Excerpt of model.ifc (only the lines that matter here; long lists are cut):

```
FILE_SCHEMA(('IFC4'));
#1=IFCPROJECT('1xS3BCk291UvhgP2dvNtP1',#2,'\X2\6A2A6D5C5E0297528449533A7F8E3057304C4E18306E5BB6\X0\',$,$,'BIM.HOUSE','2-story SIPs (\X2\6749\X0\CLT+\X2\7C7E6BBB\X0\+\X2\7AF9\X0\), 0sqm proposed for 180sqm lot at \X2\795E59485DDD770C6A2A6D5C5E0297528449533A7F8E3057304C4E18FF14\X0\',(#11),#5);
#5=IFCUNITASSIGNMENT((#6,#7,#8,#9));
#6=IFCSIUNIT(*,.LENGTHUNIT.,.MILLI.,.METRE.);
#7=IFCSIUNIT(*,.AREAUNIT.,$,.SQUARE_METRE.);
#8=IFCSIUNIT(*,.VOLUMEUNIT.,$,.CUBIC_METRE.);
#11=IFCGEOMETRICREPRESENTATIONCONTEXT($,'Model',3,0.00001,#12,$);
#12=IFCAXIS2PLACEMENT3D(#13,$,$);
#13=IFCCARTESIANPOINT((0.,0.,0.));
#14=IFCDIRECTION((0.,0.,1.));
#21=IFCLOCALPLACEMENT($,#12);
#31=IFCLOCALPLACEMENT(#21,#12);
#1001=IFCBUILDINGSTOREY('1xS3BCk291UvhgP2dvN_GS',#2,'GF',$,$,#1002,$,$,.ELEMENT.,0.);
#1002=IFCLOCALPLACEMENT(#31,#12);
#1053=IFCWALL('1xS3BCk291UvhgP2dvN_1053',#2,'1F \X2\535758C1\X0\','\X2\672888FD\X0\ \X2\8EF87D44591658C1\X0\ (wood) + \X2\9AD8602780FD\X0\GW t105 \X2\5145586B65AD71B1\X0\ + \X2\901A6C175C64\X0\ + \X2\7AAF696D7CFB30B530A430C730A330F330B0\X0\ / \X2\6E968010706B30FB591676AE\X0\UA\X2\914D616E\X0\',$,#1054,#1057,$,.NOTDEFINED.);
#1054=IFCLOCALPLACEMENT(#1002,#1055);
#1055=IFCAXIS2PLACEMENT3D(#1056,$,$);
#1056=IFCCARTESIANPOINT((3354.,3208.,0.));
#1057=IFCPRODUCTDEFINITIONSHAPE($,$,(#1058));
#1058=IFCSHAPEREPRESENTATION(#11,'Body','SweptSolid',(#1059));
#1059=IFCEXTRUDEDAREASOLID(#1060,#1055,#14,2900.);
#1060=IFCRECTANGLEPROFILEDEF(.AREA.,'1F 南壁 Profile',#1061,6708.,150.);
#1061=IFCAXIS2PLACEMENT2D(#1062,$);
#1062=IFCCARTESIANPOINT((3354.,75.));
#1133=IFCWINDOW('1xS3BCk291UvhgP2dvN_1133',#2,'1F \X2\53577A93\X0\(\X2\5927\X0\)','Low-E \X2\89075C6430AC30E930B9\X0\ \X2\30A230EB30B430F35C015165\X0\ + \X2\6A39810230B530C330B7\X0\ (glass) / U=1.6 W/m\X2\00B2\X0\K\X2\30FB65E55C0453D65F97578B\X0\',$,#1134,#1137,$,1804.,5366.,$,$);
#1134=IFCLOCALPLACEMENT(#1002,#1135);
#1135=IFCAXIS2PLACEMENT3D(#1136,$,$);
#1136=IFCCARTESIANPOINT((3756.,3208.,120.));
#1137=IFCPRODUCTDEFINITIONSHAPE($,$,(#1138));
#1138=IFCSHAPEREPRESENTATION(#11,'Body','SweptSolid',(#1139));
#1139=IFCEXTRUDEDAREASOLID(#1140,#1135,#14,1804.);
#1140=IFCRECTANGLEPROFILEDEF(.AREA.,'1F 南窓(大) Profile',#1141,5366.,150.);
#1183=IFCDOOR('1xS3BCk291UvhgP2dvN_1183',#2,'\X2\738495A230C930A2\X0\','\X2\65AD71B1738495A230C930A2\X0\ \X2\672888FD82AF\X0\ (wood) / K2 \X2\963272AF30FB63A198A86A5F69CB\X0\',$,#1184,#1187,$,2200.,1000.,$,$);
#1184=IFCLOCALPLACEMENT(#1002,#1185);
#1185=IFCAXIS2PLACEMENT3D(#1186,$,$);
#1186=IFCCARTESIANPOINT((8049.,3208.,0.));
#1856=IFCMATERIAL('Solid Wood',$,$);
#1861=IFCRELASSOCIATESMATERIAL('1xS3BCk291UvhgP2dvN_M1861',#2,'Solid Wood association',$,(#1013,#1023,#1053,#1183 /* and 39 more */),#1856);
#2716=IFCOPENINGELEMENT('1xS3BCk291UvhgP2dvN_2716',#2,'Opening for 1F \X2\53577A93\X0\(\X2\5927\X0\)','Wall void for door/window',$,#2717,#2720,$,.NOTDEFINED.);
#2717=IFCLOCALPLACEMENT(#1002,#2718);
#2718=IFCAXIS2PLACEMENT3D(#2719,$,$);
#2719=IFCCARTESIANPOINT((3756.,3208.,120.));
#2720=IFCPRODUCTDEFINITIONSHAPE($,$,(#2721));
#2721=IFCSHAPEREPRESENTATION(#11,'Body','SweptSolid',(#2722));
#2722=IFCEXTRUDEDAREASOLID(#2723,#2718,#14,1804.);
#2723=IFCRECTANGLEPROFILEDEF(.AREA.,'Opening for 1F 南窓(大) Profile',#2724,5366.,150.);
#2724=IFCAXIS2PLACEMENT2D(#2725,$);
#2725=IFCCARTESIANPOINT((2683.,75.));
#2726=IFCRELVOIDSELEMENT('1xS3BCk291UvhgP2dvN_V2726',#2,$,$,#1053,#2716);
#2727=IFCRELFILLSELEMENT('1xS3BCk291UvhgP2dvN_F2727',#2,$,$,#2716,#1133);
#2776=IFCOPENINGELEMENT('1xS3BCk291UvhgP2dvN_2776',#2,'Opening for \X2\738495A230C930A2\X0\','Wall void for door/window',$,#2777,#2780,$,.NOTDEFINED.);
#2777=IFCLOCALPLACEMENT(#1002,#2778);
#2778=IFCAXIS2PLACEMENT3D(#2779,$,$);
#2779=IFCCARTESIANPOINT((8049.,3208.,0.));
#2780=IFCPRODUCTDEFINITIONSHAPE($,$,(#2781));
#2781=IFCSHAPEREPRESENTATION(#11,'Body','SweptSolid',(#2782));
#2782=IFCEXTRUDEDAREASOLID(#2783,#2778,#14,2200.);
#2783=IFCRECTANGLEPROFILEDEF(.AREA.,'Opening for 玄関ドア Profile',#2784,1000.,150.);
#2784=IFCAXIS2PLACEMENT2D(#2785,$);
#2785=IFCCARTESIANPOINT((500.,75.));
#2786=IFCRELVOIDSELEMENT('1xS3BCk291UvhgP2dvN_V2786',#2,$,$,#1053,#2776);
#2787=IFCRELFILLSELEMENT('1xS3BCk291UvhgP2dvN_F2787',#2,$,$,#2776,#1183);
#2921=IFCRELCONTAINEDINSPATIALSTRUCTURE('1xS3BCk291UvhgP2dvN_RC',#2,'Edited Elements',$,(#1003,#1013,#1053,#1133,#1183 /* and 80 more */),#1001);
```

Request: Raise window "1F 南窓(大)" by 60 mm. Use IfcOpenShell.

```python
import numpy as np
import ifcopenshell
import ifcopenshell.api.geometry
import ifcopenshell.util.placement
import ifcopenshell.util.unit

model = ifcopenshell.open("model.ifc")
unit_scale = ifcopenshell.util.unit.calculate_unit_scale(model)

window = model.by_id(1133)
opening = window.FillsVoids[0].RelatingOpeningElement
dz = 0.06 / unit_scale

shift = np.array([0.0, 0.0, dz])
# The window is not placed relative to its opening, so move both.
for product in (opening, window):
    matrix = ifcopenshell.util.placement.get_local_placement(product.ObjectPlacement)
    matrix[:3, 3] += shift
    ifcopenshell.api.geometry.edit_object_placement(model, product=product, matrix=matrix, is_si=False)

print(f"moved by {dz * unit_scale:+.3f} m")

model.write("model-out.ifc")
```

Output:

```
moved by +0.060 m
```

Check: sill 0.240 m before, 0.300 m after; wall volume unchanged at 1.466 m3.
